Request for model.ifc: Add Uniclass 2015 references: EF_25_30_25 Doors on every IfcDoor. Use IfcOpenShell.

First a look at what the model holds.

```python
import ifcopenshell

model = ifcopenshell.open("model.ifc")
print(model.schema)
print("classifications:", [c.Name for c in model.by_type("IfcClassification")])
for ifc_class in ("IfcDoor", "IfcRoof", "IfcStair", "IfcWall", "IfcWindow"):
    print(ifc_class, len(model.by_type(ifc_class)))
```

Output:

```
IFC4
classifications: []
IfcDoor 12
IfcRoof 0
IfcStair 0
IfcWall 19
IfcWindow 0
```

```python
import ifcopenshell
import ifcopenshell.api.classification

model = ifcopenshell.open("model.ifc")

system = ifcopenshell.api.classification.add_classification(model, classification="Uniclass 2015")

codes = {
    "IfcDoor": ("EF_25_30_25", "Doors"),
}
for ifc_class, (code, name) in codes.items():
    products = model.by_type(ifc_class)
    ifcopenshell.api.classification.add_reference(
        model, products=products, classification=system, identification=code, name=name
    )
    print(code, len(products))

model.write("model_updated.ifc")
```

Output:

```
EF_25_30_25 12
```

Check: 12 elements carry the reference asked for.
